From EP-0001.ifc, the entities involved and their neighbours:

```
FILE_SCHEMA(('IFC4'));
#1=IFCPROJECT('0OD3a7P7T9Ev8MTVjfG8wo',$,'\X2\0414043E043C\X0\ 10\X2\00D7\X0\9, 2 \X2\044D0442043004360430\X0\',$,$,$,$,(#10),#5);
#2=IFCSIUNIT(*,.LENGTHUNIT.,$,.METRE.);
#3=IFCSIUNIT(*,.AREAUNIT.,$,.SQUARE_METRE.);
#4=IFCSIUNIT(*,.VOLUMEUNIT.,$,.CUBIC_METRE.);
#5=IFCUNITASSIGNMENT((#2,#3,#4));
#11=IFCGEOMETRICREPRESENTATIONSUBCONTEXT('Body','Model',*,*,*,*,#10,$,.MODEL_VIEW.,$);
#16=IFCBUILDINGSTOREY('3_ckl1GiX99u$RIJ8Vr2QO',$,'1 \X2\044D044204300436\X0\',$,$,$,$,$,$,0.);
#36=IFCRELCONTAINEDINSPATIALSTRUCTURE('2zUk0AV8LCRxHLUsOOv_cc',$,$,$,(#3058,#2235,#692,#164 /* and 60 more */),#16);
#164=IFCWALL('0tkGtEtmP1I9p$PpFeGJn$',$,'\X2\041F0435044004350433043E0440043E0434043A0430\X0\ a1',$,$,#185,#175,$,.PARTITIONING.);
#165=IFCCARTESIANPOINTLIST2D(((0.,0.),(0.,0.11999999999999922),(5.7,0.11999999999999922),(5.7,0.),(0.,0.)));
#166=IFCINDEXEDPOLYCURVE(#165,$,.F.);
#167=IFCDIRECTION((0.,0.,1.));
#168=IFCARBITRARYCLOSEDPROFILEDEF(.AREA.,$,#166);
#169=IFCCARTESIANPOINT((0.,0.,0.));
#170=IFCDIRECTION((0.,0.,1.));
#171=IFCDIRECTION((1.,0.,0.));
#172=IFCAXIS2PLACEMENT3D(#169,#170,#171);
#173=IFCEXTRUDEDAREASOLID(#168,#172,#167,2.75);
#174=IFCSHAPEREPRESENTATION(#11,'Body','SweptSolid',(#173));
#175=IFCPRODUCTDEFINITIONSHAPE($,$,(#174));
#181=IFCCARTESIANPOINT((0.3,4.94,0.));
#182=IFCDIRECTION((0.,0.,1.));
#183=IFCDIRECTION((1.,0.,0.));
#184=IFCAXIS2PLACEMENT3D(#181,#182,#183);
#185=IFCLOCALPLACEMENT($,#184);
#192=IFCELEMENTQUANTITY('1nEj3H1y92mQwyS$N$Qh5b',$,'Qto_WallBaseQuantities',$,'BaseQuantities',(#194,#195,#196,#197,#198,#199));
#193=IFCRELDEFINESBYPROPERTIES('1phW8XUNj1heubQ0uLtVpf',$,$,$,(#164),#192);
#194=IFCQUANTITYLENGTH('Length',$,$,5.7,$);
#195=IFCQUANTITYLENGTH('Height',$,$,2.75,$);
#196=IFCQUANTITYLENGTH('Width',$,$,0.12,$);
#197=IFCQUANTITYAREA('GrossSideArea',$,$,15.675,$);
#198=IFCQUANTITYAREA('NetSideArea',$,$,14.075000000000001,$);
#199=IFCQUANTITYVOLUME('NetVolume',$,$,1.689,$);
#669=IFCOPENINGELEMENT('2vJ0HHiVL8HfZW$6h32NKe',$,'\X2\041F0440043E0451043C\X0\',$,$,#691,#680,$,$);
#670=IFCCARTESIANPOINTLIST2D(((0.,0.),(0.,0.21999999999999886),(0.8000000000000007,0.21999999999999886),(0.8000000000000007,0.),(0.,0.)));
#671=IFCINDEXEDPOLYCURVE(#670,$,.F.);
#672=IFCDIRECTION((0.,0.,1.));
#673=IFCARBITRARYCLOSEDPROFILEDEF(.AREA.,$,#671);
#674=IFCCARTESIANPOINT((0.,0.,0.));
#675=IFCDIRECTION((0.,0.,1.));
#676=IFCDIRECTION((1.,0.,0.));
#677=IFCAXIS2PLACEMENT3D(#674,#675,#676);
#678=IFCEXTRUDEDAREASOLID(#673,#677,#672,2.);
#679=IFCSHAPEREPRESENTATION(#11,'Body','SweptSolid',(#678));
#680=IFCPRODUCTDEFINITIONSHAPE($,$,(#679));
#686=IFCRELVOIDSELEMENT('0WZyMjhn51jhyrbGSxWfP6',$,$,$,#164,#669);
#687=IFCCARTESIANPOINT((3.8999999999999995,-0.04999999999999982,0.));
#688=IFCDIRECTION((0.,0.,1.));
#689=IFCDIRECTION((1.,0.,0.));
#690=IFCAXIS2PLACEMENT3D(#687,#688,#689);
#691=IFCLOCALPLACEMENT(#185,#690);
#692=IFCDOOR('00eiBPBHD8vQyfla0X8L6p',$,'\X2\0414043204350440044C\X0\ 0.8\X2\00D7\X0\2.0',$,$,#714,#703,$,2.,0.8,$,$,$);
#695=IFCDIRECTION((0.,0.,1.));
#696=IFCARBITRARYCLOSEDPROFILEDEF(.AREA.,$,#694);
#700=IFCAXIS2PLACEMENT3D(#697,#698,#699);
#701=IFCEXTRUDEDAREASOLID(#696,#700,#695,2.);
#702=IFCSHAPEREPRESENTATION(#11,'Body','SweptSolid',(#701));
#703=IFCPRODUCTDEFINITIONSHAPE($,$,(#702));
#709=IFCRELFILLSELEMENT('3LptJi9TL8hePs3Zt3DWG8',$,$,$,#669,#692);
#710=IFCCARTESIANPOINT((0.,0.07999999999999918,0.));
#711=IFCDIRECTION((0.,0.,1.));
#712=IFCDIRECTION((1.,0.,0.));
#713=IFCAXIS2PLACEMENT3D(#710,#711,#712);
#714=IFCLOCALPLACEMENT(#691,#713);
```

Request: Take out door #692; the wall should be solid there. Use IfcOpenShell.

```python
import ifcopenshell
import ifcopenshell.api.feature
import ifcopenshell.api.pset
import ifcopenshell.api.root
import ifcopenshell.geom
import ifcopenshell.util.element
import ifcopenshell.util.shape
import ifcopenshell.util.unit

model = ifcopenshell.open("EP-0001.ifc")
area_scale = ifcopenshell.util.unit.calculate_unit_scale(model, "AREAUNIT")
volume_scale = ifcopenshell.util.unit.calculate_unit_scale(model, "VOLUMEUNIT")
settings = ifcopenshell.geom.settings()


def volume(element):
    """Net volume in cubic metres, openings subtracted."""
    shape = ifcopenshell.geom.create_shape(settings, element)
    return ifcopenshell.util.shape.get_volume(shape.geometry)


door = model.by_guid("00eiBPBHD8vQyfla0X8L6p")
opening = door.FillsVoids[0].RelatingOpeningElement
wall = opening.VoidsElements[0].RelatingBuildingElement
before = volume(wall)

ifcopenshell.api.root.remove_product(model, product=door)
ifcopenshell.api.feature.remove_feature(model, feature=opening)

after = volume(wall)
thickness = 0.12  # wall thickness in metres

# Update the wall's stored quantities.
qto = model.by_id(ifcopenshell.util.element.get_pset(wall, "Qto_WallBaseQuantities", should_inherit=False)["id"])
ifcopenshell.api.pset.edit_qto(model, qto=qto, properties={
    "NetSideArea": after / thickness / area_scale,
    "NetVolume": after / volume_scale,
})

print(f"wall volume {before:.3f} -> {after:.3f} m3")

model.write("EP-0001_rev.ifc")
```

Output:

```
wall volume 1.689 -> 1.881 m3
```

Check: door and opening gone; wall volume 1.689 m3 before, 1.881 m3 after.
